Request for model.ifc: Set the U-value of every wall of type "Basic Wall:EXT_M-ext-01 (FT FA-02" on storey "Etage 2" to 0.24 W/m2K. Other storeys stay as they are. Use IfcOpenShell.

First a look at what the model holds.

```python
import ifcopenshell
import ifcopenshell.util.element

model = ifcopenshell.open("model.ifc")
print(model.schema)
storey = next(s for s in model.by_type("IfcBuildingStorey") if s.Name == "Etage 2")
walls = [e for e in ifcopenshell.util.element.get_decomposition(storey) if e.is_a("IfcWall")]
seen = {}
for e in walls:
    element_type = ifcopenshell.util.element.get_type(e)
    key = (element_type.Name if element_type != e and element_type else None, ifcopenshell.util.element.get_pset(e, "Pset_WallCommon", "ThermalTransmittance"))
    seen[key] = seen.get(key, 0) + 1
for (name, value), count in sorted(seen.items(), key=str):
    print(count, "x", name, "|", value)
```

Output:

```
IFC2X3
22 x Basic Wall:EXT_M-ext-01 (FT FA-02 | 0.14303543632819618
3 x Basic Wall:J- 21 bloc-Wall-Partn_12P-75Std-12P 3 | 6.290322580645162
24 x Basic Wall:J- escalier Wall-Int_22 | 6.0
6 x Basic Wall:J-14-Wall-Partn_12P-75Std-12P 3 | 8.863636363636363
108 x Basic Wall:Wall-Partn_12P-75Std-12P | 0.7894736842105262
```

```python
import ifcopenshell
import ifcopenshell.api.pset
import ifcopenshell.util.element

model = ifcopenshell.open("model.ifc")

storey = next(s for s in model.by_type("IfcBuildingStorey") if s.Name == "Etage 2")
walls = [e for e in ifcopenshell.util.element.get_decomposition(storey) if e.is_a("IfcWall")]

count = 0
for e in walls:
    element_type = ifcopenshell.util.element.get_type(e)
    if element_type in (None, e) or element_type.Name != "Basic Wall:EXT_M-ext-01 (FT FA-02":
        continue
    # add_pset returns the element's existing set when there is one.
    pset = ifcopenshell.api.pset.add_pset(model, product=e, name="Pset_WallCommon")
    ifcopenshell.api.pset.edit_pset(model, pset=pset, properties={"ThermalTransmittance": 0.24})
    count += 1

print(count, "walls updated")

model.write("model-out.ifc")
```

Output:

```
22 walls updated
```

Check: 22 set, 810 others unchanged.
